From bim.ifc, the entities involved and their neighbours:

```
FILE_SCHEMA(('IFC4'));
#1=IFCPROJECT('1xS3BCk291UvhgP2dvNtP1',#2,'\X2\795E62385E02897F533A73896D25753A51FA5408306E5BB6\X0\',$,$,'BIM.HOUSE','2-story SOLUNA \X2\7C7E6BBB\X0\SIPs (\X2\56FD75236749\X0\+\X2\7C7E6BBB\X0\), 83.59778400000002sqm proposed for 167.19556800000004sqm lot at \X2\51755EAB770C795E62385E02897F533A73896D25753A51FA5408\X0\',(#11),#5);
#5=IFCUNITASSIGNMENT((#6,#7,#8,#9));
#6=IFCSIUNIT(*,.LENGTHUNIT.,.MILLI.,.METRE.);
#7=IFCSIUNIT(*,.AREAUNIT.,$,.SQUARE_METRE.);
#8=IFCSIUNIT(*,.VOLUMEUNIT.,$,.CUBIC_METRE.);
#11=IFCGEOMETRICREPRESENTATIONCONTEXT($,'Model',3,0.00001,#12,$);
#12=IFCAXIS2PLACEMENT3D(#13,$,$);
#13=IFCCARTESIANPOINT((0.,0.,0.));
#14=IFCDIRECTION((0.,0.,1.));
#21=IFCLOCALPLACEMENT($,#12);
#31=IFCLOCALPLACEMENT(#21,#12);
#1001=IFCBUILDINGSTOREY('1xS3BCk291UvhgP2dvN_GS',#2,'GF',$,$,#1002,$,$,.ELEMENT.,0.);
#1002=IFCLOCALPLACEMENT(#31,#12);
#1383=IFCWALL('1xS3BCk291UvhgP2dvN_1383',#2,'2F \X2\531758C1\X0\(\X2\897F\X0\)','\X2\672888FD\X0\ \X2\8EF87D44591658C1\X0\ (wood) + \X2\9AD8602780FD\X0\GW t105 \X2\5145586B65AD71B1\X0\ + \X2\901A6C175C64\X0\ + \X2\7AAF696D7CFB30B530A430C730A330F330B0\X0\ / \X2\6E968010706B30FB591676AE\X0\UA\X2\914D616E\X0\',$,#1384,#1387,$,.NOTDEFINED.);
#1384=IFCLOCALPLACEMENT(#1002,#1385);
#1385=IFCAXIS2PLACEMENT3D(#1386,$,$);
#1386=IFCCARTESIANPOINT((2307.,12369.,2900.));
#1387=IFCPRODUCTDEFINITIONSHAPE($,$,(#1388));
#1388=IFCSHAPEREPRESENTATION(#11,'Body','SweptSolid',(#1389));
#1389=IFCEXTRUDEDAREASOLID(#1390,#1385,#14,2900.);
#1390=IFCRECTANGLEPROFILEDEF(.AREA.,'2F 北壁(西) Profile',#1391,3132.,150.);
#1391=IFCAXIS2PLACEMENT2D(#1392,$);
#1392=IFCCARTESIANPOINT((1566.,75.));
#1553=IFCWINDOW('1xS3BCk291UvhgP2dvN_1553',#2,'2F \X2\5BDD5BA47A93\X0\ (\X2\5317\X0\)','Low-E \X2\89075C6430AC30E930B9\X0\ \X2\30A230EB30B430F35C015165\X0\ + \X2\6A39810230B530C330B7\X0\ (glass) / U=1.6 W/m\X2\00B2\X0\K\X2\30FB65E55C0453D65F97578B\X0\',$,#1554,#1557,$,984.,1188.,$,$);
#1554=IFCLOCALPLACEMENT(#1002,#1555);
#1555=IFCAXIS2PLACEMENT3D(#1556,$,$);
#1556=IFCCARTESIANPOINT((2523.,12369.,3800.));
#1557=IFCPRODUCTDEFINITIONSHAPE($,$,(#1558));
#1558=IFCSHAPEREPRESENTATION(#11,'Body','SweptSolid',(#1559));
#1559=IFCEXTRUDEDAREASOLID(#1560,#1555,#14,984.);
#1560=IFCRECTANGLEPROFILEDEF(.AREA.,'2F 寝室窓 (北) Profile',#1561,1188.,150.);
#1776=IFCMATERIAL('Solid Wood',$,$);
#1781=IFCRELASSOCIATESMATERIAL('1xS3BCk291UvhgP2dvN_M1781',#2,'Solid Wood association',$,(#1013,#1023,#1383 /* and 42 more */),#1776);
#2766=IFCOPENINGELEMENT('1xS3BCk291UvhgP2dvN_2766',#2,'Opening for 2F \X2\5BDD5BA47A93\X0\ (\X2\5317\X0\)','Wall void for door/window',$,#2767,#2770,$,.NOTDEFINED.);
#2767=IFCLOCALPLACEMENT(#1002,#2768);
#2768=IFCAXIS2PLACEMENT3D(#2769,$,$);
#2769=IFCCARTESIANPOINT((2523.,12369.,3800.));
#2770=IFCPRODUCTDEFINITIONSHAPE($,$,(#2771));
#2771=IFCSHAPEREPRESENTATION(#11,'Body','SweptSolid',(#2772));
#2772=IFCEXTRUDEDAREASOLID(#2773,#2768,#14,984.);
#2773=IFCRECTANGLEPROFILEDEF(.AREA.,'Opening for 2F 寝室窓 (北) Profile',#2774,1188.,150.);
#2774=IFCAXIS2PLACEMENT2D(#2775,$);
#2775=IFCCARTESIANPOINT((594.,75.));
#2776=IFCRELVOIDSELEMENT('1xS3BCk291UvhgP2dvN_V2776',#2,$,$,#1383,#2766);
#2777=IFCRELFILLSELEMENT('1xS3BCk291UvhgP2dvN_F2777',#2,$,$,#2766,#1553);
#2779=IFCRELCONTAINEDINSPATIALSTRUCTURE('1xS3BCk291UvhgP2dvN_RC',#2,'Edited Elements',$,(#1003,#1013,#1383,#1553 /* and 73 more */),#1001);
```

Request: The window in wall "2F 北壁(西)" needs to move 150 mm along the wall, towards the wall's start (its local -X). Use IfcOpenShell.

```python
import ifcopenshell
import ifcopenshell.api.geometry
import ifcopenshell.util.placement
import ifcopenshell.util.unit

model = ifcopenshell.open("bim.ifc")
unit_scale = ifcopenshell.util.unit.calculate_unit_scale(model)

window = model.by_guid("1xS3BCk291UvhgP2dvN_1553")
opening = window.FillsVoids[0].RelatingOpeningElement
wall = opening.VoidsElements[0].RelatingBuildingElement

wall_matrix = ifcopenshell.util.placement.get_local_placement(wall.ObjectPlacement)
shift = wall_matrix[:3, 0] * -0.15 / unit_scale
before = ifcopenshell.util.placement.get_local_placement(window.ObjectPlacement)[:3, 3].copy()

# The window is not placed relative to its opening, so move both.
for product in (opening, window):
    matrix = ifcopenshell.util.placement.get_local_placement(product.ObjectPlacement)
    matrix[:3, 3] += shift
    ifcopenshell.api.geometry.edit_object_placement(model, product=product, matrix=matrix, is_si=False)

after = ifcopenshell.util.placement.get_local_placement(window.ObjectPlacement)[:3, 3]
print("window moved by", (after - before).round(3) + 0.0)

model.write("bim_rev.ifc")
```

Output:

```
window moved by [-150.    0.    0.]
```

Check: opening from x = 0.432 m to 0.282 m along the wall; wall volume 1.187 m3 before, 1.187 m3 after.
